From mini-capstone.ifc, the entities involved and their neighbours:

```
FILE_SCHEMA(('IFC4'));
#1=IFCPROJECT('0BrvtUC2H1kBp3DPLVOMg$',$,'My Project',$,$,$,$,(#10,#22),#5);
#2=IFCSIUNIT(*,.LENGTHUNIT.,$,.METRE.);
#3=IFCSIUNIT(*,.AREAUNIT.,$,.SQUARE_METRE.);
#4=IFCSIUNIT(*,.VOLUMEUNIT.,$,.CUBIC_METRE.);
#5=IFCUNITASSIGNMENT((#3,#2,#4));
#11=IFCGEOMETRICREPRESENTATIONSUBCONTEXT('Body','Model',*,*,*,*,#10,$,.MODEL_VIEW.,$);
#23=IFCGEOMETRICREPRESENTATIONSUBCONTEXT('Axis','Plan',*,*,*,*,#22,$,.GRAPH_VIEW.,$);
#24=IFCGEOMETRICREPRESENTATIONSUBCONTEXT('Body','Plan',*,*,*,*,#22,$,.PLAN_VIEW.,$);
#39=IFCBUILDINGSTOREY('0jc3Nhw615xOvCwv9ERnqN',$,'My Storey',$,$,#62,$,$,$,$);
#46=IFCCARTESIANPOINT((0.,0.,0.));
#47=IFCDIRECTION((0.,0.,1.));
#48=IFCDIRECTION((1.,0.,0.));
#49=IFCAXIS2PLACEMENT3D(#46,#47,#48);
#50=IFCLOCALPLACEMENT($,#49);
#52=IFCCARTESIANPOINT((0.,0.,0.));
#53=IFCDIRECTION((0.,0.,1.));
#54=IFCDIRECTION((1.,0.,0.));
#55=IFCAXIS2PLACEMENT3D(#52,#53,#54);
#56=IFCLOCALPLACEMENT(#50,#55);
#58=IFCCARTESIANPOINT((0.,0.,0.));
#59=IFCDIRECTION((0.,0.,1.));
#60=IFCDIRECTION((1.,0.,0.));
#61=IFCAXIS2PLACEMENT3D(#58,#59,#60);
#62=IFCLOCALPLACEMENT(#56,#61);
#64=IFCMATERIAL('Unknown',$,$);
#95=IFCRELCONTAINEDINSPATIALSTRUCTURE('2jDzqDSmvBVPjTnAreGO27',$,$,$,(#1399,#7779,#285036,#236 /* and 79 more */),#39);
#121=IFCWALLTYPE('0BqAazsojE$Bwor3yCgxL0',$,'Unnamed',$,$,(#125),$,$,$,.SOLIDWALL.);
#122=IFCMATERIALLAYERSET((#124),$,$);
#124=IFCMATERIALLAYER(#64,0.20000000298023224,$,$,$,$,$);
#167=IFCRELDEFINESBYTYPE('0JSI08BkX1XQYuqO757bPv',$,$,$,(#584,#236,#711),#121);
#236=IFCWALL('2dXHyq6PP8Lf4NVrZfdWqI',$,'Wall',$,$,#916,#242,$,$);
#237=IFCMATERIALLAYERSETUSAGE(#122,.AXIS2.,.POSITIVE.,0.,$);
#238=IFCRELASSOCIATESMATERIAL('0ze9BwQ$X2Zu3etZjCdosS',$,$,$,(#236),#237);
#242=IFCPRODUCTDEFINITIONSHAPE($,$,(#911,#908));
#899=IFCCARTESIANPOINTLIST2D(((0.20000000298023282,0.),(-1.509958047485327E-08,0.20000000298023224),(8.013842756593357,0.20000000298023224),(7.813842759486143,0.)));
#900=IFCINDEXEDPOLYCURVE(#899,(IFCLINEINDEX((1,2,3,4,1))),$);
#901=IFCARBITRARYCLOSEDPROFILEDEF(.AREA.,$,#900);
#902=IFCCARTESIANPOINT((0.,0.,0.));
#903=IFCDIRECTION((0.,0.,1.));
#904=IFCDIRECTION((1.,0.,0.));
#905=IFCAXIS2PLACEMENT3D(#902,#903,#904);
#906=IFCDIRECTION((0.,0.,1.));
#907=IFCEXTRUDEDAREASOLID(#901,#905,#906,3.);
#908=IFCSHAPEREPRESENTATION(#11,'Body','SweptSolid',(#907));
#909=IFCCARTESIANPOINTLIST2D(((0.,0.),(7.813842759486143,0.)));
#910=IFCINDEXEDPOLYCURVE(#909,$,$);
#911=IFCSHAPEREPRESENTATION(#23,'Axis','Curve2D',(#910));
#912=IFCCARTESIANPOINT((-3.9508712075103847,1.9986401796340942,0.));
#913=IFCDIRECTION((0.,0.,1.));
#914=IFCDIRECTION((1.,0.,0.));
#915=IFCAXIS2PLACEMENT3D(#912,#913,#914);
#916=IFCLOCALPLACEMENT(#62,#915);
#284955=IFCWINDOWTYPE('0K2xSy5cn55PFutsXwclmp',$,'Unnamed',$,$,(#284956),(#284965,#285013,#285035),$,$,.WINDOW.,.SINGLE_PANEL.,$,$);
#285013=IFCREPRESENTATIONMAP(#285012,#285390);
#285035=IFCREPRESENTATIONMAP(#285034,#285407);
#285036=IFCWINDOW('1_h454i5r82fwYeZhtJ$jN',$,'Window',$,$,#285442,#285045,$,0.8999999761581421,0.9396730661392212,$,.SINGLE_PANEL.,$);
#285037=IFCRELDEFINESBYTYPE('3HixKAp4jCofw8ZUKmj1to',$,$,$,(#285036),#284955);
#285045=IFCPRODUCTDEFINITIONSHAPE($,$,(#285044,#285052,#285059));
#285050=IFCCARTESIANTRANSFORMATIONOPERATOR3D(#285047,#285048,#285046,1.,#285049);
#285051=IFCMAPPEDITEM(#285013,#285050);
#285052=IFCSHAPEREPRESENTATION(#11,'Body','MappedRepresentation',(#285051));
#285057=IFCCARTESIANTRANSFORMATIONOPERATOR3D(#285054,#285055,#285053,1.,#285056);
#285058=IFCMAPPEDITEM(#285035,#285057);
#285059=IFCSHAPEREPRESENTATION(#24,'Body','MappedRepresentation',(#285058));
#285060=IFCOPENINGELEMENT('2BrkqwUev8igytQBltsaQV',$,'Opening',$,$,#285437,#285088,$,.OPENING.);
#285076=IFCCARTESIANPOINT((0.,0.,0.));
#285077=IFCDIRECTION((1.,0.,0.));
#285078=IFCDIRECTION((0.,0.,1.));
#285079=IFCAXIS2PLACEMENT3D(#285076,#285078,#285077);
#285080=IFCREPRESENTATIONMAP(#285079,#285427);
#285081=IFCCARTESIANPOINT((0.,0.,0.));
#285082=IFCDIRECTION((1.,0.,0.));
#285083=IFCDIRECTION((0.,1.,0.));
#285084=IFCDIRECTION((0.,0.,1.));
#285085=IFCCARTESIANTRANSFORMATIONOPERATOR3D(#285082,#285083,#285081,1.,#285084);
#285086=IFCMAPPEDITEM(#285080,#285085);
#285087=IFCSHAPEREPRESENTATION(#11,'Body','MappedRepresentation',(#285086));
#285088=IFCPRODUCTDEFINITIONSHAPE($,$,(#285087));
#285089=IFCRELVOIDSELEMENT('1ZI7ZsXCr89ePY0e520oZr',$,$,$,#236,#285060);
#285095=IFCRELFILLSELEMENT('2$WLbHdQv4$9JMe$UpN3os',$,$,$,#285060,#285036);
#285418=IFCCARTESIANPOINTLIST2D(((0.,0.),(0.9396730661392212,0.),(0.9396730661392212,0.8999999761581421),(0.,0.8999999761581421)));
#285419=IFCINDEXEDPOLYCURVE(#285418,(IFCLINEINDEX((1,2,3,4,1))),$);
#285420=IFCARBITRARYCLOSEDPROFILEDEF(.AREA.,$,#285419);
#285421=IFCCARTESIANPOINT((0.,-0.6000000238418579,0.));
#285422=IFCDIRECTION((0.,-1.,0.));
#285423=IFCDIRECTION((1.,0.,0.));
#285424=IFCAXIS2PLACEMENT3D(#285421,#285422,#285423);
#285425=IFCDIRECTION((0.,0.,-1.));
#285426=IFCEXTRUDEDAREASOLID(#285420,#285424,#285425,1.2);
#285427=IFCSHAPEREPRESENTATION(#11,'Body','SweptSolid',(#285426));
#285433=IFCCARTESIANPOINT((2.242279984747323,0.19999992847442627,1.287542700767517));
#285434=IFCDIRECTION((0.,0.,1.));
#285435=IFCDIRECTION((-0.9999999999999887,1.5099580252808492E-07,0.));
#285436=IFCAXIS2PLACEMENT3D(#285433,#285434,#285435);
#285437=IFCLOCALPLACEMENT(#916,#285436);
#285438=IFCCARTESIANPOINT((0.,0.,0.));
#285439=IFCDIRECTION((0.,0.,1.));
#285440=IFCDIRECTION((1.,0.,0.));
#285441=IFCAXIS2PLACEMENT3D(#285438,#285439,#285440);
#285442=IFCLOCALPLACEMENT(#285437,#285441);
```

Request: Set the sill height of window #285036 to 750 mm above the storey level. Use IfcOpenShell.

```python
import numpy as np
import ifcopenshell
import ifcopenshell.api.geometry
import ifcopenshell.geom
import ifcopenshell.util.element
import ifcopenshell.util.placement
import ifcopenshell.util.shape
import ifcopenshell.util.unit

model = ifcopenshell.open("mini-capstone.ifc")
unit_scale = ifcopenshell.util.unit.calculate_unit_scale(model)

window = model.by_guid("1_h454i5r82fwYeZhtJ$jN")
opening = window.FillsVoids[0].RelatingOpeningElement
storey = ifcopenshell.util.element.get_container(window, ifc_class="IfcBuildingStorey")
level = ifcopenshell.util.placement.get_local_placement(storey.ObjectPlacement)[2, 3]

# The opening's origin need not be at the sill, so measure its lowest point.
shape = ifcopenshell.geom.create_shape(ifcopenshell.geom.settings(), opening)
bottom = ifcopenshell.util.shape.get_shape_bottom_elevation(shape, shape.geometry) / unit_scale
dz = level + 0.75 / unit_scale - bottom

shift = np.array([0.0, 0.0, dz])
# The window is placed relative to its opening, so it follows when the opening moves.
matrix = ifcopenshell.util.placement.get_local_placement(opening.ObjectPlacement)
matrix[:3, 3] += shift
ifcopenshell.api.geometry.edit_object_placement(
    model, product=opening, matrix=matrix, is_si=False, should_transform_children=True
)

print(f"moved by {dz * unit_scale:+.3f} m")

model.write("mini-capstone-out.ifc")
```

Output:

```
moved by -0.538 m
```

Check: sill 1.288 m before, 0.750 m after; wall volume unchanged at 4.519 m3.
